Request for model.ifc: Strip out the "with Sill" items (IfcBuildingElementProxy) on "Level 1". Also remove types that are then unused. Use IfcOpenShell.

First a look at what the model holds.

```python
import ifcopenshell
import ifcopenshell.util.element

model = ifcopenshell.open("model.ifc")
print(model.schema)
storey = next(s for s in model.by_type("IfcBuildingStorey") if s.Name == "Level 1")
proxies = [e for e in ifcopenshell.util.element.get_decomposition(storey) if e.is_a("IfcBuildingElementProxy")]
seen = {}
for e in proxies:
    element_type = ifcopenshell.util.element.get_type(e)
    name = element_type.Name if element_type not in (None, e) else None
    seen[name] = seen.get(name, 0) + 1
for name, count in sorted(seen.items(), key=str):
    print(count, "x", name)
```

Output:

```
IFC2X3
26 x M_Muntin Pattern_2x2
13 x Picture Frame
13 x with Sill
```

```python
import ifcopenshell
import ifcopenshell.api.root
import ifcopenshell.util.element

model = ifcopenshell.open("model.ifc")

storey = next(s for s in model.by_type("IfcBuildingStorey") if s.Name == "Level 1")
proxies = [e for e in ifcopenshell.util.element.get_decomposition(storey) if e.is_a("IfcBuildingElementProxy")]
targets = [e for e in proxies if (t := ifcopenshell.util.element.get_type(e)) not in (None, e) and t.Name == "with Sill"]
types = {ifcopenshell.util.element.get_type(e) for e in targets} - {None, *targets}

for e in targets:
    ifcopenshell.api.root.remove_product(model, product=e)
print(len(targets), "removed")

unused = [t for t in types if not ifcopenshell.util.element.get_types(t)]
for t in unused:
    ifcopenshell.api.root.remove_product(model, product=t)
print(len(unused), "unused types removed")

model.write("model_edited.ifc")
```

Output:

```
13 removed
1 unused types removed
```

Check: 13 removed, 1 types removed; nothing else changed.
